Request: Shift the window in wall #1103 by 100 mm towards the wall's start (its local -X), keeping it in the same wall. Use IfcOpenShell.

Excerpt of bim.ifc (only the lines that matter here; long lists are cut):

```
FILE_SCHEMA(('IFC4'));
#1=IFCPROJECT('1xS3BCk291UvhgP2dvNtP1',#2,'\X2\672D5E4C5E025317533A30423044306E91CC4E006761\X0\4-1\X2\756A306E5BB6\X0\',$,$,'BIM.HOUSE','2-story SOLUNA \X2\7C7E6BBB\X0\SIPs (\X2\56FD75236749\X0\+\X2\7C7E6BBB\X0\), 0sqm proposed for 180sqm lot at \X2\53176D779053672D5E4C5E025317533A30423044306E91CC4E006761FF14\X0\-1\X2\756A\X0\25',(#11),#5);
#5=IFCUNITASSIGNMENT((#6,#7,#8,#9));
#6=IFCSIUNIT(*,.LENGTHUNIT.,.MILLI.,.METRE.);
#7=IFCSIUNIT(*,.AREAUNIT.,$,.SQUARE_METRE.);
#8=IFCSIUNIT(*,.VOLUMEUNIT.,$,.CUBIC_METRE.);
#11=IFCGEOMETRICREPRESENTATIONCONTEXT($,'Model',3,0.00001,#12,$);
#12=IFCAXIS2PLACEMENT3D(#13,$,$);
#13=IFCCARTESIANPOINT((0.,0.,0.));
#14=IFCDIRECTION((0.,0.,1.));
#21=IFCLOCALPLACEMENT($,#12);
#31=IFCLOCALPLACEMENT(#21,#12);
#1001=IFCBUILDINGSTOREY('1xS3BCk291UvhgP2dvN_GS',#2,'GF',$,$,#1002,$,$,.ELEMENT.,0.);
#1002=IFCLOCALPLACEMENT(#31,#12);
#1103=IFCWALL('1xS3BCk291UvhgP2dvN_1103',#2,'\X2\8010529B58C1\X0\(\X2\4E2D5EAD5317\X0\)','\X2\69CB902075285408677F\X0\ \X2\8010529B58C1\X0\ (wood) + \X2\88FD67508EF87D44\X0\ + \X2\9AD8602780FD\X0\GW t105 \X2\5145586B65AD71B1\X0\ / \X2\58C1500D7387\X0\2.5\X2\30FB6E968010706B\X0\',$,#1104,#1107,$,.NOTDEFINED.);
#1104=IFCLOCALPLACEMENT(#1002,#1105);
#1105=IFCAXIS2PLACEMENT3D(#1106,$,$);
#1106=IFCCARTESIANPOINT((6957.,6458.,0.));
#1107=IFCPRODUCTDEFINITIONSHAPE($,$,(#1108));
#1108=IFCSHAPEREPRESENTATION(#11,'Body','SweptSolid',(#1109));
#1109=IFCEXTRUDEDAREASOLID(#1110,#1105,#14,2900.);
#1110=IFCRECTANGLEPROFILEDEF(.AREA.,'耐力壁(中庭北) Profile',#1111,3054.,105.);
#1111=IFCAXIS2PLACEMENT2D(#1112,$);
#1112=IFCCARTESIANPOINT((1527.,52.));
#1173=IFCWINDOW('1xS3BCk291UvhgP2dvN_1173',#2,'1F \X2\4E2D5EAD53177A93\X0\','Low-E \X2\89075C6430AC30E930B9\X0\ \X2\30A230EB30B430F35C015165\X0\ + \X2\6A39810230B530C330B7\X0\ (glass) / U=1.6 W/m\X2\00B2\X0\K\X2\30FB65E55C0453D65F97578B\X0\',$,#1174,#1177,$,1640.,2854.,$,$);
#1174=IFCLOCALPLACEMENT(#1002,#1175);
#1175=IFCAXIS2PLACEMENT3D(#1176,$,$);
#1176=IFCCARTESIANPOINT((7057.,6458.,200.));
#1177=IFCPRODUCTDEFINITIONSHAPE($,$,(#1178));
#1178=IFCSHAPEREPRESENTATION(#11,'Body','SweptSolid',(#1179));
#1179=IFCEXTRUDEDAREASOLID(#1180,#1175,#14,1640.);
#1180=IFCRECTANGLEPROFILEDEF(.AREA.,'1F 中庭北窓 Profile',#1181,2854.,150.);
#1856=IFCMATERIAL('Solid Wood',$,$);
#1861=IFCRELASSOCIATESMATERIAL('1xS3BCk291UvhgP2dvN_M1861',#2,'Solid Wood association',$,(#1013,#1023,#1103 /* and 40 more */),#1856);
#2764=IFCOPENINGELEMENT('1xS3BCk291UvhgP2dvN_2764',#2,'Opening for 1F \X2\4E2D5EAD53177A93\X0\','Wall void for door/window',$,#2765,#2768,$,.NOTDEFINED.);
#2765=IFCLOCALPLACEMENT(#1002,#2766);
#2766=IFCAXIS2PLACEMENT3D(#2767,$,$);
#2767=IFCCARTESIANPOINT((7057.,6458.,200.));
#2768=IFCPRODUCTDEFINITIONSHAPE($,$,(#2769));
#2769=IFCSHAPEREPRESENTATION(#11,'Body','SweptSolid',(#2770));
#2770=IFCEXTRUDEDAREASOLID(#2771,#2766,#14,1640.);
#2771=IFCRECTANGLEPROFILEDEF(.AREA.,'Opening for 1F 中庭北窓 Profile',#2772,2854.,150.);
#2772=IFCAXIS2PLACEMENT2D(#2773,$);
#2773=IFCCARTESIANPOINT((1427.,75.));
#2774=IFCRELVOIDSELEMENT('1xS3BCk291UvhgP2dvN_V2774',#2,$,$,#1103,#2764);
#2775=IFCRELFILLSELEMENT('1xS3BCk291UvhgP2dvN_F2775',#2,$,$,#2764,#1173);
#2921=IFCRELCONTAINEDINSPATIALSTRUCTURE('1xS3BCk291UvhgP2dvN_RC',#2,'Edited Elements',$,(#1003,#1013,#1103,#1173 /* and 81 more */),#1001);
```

```python
import ifcopenshell
import ifcopenshell.api.geometry
import ifcopenshell.util.placement
import ifcopenshell.util.unit

model = ifcopenshell.open("bim.ifc")
unit_scale = ifcopenshell.util.unit.calculate_unit_scale(model)

window = model.by_guid("1xS3BCk291UvhgP2dvN_1173")
opening = window.FillsVoids[0].RelatingOpeningElement
wall = opening.VoidsElements[0].RelatingBuildingElement

wall_matrix = ifcopenshell.util.placement.get_local_placement(wall.ObjectPlacement)
shift = wall_matrix[:3, 0] * -0.1 / unit_scale
before = ifcopenshell.util.placement.get_local_placement(window.ObjectPlacement)[:3, 3].copy()

# The window is not placed relative to its opening, so move both.
for product in (opening, window):
    matrix = ifcopenshell.util.placement.get_local_placement(product.ObjectPlacement)
    matrix[:3, 3] += shift
    ifcopenshell.api.geometry.edit_object_placement(model, product=product, matrix=matrix, is_si=False)

after = ifcopenshell.util.placement.get_local_placement(window.ObjectPlacement)[:3, 3]
print("window moved by", (after - before).round(3) + 0.0)

model.write("bim_v2.ifc")
```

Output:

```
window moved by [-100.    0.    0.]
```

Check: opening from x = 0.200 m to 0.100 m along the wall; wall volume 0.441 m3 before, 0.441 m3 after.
